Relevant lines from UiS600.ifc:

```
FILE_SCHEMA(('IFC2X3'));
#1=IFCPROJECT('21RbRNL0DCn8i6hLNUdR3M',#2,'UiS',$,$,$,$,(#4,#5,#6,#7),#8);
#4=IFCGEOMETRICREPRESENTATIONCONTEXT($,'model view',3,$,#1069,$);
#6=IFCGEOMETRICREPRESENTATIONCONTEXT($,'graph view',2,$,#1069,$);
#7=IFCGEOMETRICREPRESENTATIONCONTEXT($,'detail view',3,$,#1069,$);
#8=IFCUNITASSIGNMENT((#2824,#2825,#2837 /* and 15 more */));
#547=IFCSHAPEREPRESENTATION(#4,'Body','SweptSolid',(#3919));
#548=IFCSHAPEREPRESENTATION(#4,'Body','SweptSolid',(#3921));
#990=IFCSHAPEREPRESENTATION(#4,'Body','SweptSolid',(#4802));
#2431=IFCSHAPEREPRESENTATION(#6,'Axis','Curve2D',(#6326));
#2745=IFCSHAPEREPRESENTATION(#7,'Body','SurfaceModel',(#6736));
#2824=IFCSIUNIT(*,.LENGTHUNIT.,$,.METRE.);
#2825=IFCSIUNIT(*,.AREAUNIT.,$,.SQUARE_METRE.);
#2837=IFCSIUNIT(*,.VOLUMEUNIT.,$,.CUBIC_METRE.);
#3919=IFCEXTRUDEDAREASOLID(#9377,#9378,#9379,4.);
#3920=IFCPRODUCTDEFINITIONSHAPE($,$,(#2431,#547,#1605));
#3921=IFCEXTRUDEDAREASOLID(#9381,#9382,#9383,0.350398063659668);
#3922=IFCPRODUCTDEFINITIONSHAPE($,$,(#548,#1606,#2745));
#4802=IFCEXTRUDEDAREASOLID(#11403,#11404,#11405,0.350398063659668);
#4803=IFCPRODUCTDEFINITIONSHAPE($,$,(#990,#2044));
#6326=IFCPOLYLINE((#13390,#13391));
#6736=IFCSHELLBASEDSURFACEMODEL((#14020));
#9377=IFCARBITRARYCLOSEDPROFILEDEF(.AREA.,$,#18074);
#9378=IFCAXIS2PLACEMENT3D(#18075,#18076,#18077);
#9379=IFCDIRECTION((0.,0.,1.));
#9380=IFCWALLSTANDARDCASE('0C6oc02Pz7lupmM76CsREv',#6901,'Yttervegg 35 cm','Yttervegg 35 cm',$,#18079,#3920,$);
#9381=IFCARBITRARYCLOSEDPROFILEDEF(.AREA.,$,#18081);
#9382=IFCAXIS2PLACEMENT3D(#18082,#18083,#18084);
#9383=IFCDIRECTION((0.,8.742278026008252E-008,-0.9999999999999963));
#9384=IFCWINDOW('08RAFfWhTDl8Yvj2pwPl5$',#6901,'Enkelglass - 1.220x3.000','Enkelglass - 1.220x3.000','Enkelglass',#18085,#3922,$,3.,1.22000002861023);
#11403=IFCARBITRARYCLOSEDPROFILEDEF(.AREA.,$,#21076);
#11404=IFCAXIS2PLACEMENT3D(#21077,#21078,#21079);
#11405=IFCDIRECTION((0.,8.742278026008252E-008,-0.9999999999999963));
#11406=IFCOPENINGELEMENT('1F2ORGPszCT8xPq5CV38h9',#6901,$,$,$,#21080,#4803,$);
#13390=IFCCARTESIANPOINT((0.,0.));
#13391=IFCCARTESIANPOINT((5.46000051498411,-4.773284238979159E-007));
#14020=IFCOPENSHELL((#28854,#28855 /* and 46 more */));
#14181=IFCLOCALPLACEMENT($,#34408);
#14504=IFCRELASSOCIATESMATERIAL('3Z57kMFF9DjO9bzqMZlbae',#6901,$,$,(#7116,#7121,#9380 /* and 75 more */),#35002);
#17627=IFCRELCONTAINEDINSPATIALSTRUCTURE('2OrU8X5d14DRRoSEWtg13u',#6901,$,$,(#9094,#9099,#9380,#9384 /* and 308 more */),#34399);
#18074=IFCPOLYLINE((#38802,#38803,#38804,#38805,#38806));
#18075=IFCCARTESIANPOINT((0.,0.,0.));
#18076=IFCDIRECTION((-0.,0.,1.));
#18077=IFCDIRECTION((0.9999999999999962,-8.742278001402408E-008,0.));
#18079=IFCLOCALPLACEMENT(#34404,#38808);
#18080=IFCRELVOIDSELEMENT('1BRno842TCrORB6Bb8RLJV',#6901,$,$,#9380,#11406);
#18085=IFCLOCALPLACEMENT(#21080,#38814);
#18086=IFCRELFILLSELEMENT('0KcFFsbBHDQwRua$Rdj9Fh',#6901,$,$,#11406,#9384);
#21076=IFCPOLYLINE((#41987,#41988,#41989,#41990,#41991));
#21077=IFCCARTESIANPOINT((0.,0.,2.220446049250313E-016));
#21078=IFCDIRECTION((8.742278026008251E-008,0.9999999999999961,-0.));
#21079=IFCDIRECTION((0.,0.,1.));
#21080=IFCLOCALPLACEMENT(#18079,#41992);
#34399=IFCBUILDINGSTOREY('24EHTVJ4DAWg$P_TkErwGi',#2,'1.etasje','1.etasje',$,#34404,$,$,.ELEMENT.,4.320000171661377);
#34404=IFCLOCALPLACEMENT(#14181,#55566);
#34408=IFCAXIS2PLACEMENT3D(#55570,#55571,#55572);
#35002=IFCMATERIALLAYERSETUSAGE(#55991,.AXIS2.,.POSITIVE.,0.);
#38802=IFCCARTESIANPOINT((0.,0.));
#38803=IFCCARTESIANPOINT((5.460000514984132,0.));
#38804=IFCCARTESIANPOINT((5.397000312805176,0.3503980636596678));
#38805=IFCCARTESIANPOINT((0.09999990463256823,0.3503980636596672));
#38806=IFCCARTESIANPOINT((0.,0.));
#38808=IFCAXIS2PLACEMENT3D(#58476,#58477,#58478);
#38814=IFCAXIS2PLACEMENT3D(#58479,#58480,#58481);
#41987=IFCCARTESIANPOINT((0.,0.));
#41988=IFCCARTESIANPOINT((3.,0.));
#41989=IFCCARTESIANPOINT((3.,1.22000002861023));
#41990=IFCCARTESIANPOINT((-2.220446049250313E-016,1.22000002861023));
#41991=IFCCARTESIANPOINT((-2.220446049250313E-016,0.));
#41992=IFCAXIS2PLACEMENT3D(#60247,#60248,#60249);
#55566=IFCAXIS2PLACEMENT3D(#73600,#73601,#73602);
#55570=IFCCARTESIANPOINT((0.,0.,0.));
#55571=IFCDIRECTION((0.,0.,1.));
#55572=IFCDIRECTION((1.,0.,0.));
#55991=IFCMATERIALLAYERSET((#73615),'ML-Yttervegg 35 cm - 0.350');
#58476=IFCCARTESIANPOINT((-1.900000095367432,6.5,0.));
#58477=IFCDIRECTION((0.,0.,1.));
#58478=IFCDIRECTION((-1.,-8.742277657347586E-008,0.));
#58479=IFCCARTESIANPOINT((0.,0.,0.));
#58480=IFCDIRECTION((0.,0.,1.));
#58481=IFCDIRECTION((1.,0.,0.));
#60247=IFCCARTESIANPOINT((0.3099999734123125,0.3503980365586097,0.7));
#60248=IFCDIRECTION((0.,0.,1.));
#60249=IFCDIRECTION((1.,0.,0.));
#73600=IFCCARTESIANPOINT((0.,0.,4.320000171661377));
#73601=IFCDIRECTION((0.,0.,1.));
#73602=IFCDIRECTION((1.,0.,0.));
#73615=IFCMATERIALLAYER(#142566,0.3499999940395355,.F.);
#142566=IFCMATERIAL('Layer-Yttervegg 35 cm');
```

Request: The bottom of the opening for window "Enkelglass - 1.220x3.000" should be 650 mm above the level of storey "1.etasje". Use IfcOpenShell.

```python
import numpy as np
import ifcopenshell
import ifcopenshell.api.geometry
import ifcopenshell.geom
import ifcopenshell.util.element
import ifcopenshell.util.placement
import ifcopenshell.util.shape
import ifcopenshell.util.unit

model = ifcopenshell.open("UiS600.ifc")
unit_scale = ifcopenshell.util.unit.calculate_unit_scale(model)

window = model.by_guid("08RAFfWhTDl8Yvj2pwPl5$")
opening = window.FillsVoids[0].RelatingOpeningElement
storey = ifcopenshell.util.element.get_container(window, ifc_class="IfcBuildingStorey")
level = ifcopenshell.util.placement.get_local_placement(storey.ObjectPlacement)[2, 3]

# The opening's origin need not be at the sill, so measure its lowest point.
shape = ifcopenshell.geom.create_shape(ifcopenshell.geom.settings(), opening)
bottom = ifcopenshell.util.shape.get_shape_bottom_elevation(shape, shape.geometry) / unit_scale
dz = level + 0.65 - bottom

shift = np.array([0.0, 0.0, dz])
# The window is placed relative to its opening, so it follows when the opening moves.
matrix = ifcopenshell.util.placement.get_local_placement(opening.ObjectPlacement)
matrix[:3, 3] += shift
ifcopenshell.api.geometry.edit_object_placement(
    model, product=opening, matrix=matrix, is_si=False, should_transform_children=True
)

print(f"moved by {dz * unit_scale:+.3f} m")

model.write("UiS600_rev.ifc")
```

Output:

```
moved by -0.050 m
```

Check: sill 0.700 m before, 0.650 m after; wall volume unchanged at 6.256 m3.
